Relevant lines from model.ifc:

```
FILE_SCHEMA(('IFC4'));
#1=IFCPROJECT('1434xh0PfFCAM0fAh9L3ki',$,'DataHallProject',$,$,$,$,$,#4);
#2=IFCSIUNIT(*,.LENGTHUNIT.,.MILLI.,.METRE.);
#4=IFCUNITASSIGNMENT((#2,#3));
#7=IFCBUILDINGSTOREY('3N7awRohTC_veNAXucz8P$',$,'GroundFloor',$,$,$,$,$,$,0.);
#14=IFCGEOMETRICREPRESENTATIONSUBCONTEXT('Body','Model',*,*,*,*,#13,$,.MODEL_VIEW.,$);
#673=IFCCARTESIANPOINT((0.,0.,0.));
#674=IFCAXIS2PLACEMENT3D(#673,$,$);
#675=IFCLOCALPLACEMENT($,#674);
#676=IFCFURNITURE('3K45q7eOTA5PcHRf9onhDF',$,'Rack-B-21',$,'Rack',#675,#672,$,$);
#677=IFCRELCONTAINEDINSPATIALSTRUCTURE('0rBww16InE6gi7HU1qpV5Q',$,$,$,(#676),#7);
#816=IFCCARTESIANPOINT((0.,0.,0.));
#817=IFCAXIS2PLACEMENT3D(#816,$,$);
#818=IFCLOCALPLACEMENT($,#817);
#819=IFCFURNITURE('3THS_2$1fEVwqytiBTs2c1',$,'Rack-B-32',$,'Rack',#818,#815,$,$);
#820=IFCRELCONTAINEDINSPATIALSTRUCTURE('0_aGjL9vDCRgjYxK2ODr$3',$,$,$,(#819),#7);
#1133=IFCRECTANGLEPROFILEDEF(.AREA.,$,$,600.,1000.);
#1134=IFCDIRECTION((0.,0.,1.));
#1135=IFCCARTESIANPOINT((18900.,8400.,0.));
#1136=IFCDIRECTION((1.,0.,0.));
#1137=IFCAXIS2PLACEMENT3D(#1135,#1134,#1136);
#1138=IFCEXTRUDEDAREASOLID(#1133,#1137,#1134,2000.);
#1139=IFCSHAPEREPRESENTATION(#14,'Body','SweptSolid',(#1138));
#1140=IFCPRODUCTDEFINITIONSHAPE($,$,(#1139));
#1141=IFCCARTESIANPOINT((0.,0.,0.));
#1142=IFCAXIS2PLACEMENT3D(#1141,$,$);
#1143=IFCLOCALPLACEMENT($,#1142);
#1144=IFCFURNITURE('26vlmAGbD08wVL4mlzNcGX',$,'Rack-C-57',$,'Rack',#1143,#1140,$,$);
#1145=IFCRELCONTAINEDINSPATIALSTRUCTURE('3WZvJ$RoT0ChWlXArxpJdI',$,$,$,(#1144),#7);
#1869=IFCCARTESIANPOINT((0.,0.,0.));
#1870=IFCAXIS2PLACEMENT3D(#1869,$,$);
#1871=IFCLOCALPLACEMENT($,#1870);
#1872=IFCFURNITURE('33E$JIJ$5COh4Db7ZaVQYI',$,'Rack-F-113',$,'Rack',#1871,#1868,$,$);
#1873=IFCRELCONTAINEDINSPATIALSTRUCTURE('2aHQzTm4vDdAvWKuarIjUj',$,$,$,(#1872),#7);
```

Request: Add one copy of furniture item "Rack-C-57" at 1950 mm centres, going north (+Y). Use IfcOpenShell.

```python
import numpy as np
import ifcopenshell
import ifcopenshell.api.geometry
import ifcopenshell.api.root
import ifcopenshell.util.element
import ifcopenshell.util.placement
import ifcopenshell.util.unit

model = ifcopenshell.open("model.ifc")
unit_scale = ifcopenshell.util.unit.calculate_unit_scale(model)

source = model.by_id(1144)
base = ifcopenshell.util.placement.get_local_placement(source.ObjectPlacement)
step = np.array([0.0, 1.0, 0.0]) * 1.95 / unit_scale

for i in range(1, 2):
    copy = ifcopenshell.api.root.copy_class(model, product=source)
    copy.Representation = ifcopenshell.util.element.copy_deep(
        model, source.Representation, exclude=["IfcGeometricRepresentationContext", "IfcRepresentationMap"]
    )
    matrix = base.copy()
    matrix[:3, 3] += i * step
    print("added at", matrix[:3, 3].round(3) + 0.0)
    ifcopenshell.api.geometry.edit_object_placement(model, product=copy, matrix=matrix, is_si=False)

model.write("model_edited.ifc")
```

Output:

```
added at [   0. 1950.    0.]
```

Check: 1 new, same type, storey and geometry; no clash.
